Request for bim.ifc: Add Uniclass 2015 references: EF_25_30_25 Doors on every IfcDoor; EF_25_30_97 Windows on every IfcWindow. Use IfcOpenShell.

First a look at what the model holds.

```python
import ifcopenshell

model = ifcopenshell.open("bim.ifc")
print(model.schema)
print("classifications:", [c.Name for c in model.by_type("IfcClassification")])
for ifc_class in ("IfcDoor", "IfcRoof", "IfcStair", "IfcWall", "IfcWindow"):
    print(ifc_class, len(model.by_type(ifc_class)))
```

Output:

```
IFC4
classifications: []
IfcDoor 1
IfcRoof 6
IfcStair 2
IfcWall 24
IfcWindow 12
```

```python
import ifcopenshell
import ifcopenshell.api.classification

model = ifcopenshell.open("bim.ifc")

system = ifcopenshell.api.classification.add_classification(model, classification="Uniclass 2015")

codes = {
    "IfcDoor": ("EF_25_30_25", "Doors"),
    "IfcWindow": ("EF_25_30_97", "Windows"),
}
for ifc_class, (code, name) in codes.items():
    products = model.by_type(ifc_class)
    ifcopenshell.api.classification.add_reference(
        model, products=products, classification=system, identification=code, name=name
    )
    print(code, len(products))

model.write("bim_rev.ifc")
```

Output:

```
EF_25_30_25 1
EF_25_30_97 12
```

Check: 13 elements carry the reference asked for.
